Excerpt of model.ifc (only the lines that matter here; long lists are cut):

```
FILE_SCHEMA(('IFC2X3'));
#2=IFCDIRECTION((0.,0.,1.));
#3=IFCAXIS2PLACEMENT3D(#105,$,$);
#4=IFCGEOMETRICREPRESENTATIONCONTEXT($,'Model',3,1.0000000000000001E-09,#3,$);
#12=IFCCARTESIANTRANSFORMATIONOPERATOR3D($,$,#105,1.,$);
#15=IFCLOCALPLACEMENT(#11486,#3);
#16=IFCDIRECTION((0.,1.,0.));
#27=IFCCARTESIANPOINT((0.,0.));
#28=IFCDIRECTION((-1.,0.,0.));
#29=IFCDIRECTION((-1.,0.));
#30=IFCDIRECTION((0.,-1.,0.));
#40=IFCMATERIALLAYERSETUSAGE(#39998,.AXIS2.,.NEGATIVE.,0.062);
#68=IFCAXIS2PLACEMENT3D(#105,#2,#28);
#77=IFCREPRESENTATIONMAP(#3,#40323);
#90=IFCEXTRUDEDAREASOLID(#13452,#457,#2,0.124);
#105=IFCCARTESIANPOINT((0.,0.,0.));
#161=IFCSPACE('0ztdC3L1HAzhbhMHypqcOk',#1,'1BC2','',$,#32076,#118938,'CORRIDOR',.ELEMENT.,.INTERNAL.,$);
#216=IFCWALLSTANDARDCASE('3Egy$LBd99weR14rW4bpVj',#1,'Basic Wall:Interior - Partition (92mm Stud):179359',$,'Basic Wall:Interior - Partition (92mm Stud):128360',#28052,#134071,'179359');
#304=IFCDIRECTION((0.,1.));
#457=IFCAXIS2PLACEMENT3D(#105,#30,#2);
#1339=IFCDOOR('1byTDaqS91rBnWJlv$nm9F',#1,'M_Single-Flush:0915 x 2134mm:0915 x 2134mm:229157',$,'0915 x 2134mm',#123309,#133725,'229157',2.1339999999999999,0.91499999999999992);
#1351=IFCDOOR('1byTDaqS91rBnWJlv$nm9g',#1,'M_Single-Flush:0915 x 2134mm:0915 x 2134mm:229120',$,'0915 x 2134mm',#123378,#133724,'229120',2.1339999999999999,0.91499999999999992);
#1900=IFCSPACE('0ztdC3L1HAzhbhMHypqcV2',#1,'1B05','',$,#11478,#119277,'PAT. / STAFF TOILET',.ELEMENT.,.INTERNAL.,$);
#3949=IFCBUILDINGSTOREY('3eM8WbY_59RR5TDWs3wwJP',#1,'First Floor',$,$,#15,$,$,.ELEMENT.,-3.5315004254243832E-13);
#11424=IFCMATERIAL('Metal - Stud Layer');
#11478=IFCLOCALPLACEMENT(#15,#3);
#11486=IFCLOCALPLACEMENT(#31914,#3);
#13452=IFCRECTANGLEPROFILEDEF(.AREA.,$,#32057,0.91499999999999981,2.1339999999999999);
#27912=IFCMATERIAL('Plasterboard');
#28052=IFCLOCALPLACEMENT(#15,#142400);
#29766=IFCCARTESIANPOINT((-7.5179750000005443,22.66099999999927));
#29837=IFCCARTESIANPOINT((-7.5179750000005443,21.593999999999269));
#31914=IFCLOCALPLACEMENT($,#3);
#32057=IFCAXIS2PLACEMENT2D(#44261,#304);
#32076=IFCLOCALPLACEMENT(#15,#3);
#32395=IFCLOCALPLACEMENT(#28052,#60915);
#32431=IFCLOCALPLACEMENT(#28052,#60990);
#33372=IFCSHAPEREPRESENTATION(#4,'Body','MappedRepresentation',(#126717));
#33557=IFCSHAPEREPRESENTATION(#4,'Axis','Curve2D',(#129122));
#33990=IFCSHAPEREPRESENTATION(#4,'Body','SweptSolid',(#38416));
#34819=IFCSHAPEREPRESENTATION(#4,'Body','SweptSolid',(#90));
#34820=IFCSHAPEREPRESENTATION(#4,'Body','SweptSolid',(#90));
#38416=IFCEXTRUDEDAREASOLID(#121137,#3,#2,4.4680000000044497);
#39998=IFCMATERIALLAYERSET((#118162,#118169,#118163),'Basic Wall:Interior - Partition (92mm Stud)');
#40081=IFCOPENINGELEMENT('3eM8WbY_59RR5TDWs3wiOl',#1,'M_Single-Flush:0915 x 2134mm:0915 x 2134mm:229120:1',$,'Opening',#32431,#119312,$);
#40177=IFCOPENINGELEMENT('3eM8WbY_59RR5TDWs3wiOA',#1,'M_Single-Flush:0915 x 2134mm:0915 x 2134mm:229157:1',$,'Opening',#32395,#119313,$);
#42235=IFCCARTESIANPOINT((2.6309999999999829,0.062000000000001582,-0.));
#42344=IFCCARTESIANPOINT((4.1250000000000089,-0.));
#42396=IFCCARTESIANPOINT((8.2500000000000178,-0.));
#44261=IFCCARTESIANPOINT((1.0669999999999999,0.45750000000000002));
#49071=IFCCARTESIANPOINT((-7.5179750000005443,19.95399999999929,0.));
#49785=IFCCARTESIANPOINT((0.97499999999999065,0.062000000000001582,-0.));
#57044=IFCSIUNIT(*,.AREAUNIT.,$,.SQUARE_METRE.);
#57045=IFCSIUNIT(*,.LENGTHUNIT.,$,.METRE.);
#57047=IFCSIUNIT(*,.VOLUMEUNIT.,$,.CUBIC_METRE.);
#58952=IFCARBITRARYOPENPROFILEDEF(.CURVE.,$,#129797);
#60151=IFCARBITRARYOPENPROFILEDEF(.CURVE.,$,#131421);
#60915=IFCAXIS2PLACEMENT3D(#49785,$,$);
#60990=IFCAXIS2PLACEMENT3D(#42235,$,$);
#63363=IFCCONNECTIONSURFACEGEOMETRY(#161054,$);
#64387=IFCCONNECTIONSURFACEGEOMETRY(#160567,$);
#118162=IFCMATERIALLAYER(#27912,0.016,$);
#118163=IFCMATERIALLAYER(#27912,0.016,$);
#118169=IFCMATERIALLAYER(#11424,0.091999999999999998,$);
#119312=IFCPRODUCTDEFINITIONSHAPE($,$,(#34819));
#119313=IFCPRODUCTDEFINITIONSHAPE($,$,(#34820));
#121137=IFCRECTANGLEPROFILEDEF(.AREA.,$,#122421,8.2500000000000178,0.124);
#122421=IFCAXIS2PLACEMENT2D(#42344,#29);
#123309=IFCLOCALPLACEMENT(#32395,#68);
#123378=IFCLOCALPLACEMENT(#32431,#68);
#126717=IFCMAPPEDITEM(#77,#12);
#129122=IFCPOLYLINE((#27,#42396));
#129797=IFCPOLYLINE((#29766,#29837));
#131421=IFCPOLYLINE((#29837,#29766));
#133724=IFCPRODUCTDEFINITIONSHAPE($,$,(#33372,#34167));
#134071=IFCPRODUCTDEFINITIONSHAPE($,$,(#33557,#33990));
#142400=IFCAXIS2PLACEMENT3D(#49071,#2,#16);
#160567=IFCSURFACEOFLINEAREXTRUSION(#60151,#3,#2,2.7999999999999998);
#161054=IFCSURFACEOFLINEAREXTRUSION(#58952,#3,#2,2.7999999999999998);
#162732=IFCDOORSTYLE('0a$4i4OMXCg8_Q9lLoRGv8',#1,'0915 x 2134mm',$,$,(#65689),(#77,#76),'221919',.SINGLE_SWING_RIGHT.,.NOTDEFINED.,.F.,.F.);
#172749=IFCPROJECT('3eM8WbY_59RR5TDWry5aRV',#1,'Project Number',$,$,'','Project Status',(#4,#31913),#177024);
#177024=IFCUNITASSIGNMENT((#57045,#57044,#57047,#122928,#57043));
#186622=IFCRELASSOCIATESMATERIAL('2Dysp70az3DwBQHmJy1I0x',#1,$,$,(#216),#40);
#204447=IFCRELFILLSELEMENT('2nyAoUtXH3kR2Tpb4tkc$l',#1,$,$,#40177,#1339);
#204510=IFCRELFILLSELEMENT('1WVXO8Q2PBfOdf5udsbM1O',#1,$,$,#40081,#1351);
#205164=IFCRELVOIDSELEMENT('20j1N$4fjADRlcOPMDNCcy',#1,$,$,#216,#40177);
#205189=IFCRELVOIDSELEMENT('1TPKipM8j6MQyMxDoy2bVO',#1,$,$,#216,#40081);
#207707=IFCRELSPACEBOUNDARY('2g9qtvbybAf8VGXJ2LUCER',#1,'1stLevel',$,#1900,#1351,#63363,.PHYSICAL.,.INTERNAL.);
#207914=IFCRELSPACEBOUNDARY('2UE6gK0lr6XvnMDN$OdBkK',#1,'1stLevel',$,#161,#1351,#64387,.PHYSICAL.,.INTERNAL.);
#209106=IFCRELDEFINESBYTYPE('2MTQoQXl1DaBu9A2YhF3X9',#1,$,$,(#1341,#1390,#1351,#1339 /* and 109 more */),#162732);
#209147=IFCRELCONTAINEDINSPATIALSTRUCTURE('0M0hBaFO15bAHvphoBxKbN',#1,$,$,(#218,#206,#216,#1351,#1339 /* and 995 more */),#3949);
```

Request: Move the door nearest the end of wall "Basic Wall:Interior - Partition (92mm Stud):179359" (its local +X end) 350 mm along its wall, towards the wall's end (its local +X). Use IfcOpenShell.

```python
import numpy as np
import ifcopenshell
import ifcopenshell.api.geometry
import ifcopenshell.util.placement

model = ifcopenshell.open("model.ifc")

door = model.by_guid("1byTDaqS91rBnWJlv$nm9g")
opening = door.FillsVoids[0].RelatingOpeningElement
wall = opening.VoidsElements[0].RelatingBuildingElement

wall_matrix = ifcopenshell.util.placement.get_local_placement(wall.ObjectPlacement)
shift = wall_matrix[:3, 0] * 0.35
before = ifcopenshell.util.placement.get_local_placement(door.ObjectPlacement)[:3, 3].copy()

# The door is placed relative to its opening, so it follows when the opening moves.
matrix = ifcopenshell.util.placement.get_local_placement(opening.ObjectPlacement)
matrix[:3, 3] += shift
ifcopenshell.api.geometry.edit_object_placement(
    model, product=opening, matrix=matrix, is_si=False, should_transform_children=True
)

# Space boundary surfaces are stored in each space's coordinates; move them too.
for rel in door.ProvidesBoundaries:
    if not rel.ConnectionGeometry:
        continue
    surface = rel.ConnectionGeometry.SurfaceOnRelatingElement
    space_matrix = ifcopenshell.util.placement.get_local_placement(rel.RelatingSpace.ObjectPlacement)
    point = np.array(surface.Position.Location.Coordinates) + space_matrix[:3, :3].T @ shift
    surface.Position = model.createIfcAxis2Placement3D(
        model.createIfcCartesianPoint(point.tolist()), surface.Position.Axis, surface.Position.RefDirection
    )

after = ifcopenshell.util.placement.get_local_placement(door.ObjectPlacement)[:3, 3]
print("door moved by", (after - before).round(3) + 0.0)

model.write("model_rev.ifc")
```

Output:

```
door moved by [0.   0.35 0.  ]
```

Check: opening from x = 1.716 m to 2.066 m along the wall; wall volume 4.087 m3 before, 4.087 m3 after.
